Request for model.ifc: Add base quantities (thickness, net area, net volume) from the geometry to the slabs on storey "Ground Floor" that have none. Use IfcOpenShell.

First a look at what the model holds.

```python
import ifcopenshell
import ifcopenshell.util.element
import ifcopenshell.util.unit

model = ifcopenshell.open("model.ifc")
print(model.schema)
for unit_type in ("LENGTHUNIT", "AREAUNIT", "VOLUMEUNIT"):
    print(unit_type, ifcopenshell.util.unit.calculate_unit_scale(model, unit_type))
storey = next(s for s in model.by_type("IfcBuildingStorey") if s.Name == "Ground Floor")
slabs = [e for e in ifcopenshell.util.element.get_decomposition(storey) if e.is_a("IfcSlab")]
for e in sorted(slabs, key=lambda e: e.id()):
    print(e.id(), e.is_a(), e.Name, list(ifcopenshell.util.element.get_psets(e, qtos_only=True)), sep=" | ")
```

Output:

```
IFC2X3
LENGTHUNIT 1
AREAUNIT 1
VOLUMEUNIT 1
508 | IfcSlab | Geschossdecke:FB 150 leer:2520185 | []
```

```python
import ifcopenshell
import ifcopenshell.api.pset
import ifcopenshell.geom
import ifcopenshell.util.element
import ifcopenshell.util.shape
import ifcopenshell.util.unit

model = ifcopenshell.open("model.ifc")
unit_scale = ifcopenshell.util.unit.calculate_unit_scale(model)
area_scale = ifcopenshell.util.unit.calculate_unit_scale(model, "AREAUNIT")
volume_scale = ifcopenshell.util.unit.calculate_unit_scale(model, "VOLUMEUNIT")
settings = ifcopenshell.geom.settings()

storey = next(s for s in model.by_type("IfcBuildingStorey") if s.Name == "Ground Floor")
slabs = [e for e in ifcopenshell.util.element.get_decomposition(storey) if e.is_a("IfcSlab")]

for e in sorted(slabs, key=lambda e: e.id()):
    if ifcopenshell.util.element.get_psets(e, qtos_only=True, should_inherit=False):
        continue
    # Geometry comes back in metres, in the element's own axes.
    shape = ifcopenshell.geom.create_shape(settings, e)
    values = {
        "Width": ifcopenshell.util.shape.get_z(shape.geometry) / unit_scale,
        "NetArea": ifcopenshell.util.shape.get_footprint_area(shape.geometry) / area_scale,
        "NetVolume": ifcopenshell.util.shape.get_volume(shape.geometry) / volume_scale,
    }
    qto = ifcopenshell.api.pset.add_qto(model, product=e, name="BaseQuantities")
    ifcopenshell.api.pset.edit_qto(model, qto=qto, properties=values)
    print(e.id(), {k: round(v, 3) for k, v in values.items()})

model.write("model_v2.ifc")
```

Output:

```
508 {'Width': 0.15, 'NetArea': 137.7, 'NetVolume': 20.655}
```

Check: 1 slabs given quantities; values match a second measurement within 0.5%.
